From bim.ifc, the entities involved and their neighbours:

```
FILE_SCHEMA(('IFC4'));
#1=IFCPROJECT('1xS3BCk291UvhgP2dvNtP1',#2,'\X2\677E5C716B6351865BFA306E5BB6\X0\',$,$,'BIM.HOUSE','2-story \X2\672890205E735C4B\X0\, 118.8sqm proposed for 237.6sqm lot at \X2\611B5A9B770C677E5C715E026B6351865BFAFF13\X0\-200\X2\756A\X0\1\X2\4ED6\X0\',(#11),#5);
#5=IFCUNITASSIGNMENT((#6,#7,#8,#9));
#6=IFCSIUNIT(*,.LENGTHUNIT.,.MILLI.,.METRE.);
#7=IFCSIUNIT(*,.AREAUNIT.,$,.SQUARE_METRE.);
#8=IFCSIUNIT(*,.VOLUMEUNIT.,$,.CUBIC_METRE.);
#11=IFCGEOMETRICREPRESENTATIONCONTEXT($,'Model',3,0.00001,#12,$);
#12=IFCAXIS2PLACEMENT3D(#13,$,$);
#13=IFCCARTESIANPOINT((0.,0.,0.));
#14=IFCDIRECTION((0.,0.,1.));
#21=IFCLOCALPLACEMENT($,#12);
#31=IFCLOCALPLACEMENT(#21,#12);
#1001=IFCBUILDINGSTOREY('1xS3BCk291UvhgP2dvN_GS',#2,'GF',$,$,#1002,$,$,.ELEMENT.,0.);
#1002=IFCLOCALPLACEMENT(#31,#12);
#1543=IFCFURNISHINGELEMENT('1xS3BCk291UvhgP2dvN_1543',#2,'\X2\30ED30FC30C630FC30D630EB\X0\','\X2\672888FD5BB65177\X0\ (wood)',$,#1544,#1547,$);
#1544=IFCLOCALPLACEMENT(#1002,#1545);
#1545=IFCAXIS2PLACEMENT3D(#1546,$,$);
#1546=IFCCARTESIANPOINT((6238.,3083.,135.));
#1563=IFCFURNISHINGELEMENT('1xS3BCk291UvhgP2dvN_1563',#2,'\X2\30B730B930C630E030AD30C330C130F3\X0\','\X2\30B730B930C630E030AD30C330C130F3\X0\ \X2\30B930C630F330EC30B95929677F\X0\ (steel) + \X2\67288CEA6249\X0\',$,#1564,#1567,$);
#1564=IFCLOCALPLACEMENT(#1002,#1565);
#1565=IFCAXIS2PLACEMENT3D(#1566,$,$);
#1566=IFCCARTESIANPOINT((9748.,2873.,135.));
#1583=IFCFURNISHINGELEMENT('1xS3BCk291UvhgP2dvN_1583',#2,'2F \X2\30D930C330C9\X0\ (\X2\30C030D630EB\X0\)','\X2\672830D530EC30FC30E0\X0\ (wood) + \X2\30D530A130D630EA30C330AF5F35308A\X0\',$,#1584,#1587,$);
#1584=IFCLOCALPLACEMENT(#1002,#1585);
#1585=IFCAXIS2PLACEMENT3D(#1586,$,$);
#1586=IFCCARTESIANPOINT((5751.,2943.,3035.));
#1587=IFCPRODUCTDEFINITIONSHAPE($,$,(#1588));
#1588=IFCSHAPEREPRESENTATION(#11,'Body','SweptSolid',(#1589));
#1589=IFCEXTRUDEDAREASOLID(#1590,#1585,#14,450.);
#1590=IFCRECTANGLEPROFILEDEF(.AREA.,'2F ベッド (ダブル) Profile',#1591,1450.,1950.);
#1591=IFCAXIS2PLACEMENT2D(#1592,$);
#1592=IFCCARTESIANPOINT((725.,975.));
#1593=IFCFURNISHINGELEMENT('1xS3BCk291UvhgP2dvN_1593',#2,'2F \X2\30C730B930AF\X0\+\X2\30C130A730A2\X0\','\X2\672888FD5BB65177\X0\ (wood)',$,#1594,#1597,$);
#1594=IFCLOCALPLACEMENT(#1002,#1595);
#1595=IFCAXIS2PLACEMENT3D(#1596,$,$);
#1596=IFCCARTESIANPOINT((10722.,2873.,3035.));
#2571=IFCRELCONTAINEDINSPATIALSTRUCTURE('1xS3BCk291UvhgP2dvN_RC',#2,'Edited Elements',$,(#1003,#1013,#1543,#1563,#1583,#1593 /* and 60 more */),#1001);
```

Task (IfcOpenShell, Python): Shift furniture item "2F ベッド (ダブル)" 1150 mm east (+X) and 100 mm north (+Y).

```python
import ifcopenshell
import ifcopenshell.api.geometry
import ifcopenshell.util.placement

model = ifcopenshell.open("bim.ifc")

item = model.by_guid("1xS3BCk291UvhgP2dvN_1583")
matrix = ifcopenshell.util.placement.get_local_placement(item.ObjectPlacement)
matrix[0, 3] += 1150.0
matrix[1, 3] += 100.0
ifcopenshell.api.geometry.edit_object_placement(model, product=item, matrix=matrix, is_si=False)

print(ifcopenshell.util.placement.get_local_placement(item.ObjectPlacement).round(3) + 0.0)

model.write("bim_updated.ifc")
```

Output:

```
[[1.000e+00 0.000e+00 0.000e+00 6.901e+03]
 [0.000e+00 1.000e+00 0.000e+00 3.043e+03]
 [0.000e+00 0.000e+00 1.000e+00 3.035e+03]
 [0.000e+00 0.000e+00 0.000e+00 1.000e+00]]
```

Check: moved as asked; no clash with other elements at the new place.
